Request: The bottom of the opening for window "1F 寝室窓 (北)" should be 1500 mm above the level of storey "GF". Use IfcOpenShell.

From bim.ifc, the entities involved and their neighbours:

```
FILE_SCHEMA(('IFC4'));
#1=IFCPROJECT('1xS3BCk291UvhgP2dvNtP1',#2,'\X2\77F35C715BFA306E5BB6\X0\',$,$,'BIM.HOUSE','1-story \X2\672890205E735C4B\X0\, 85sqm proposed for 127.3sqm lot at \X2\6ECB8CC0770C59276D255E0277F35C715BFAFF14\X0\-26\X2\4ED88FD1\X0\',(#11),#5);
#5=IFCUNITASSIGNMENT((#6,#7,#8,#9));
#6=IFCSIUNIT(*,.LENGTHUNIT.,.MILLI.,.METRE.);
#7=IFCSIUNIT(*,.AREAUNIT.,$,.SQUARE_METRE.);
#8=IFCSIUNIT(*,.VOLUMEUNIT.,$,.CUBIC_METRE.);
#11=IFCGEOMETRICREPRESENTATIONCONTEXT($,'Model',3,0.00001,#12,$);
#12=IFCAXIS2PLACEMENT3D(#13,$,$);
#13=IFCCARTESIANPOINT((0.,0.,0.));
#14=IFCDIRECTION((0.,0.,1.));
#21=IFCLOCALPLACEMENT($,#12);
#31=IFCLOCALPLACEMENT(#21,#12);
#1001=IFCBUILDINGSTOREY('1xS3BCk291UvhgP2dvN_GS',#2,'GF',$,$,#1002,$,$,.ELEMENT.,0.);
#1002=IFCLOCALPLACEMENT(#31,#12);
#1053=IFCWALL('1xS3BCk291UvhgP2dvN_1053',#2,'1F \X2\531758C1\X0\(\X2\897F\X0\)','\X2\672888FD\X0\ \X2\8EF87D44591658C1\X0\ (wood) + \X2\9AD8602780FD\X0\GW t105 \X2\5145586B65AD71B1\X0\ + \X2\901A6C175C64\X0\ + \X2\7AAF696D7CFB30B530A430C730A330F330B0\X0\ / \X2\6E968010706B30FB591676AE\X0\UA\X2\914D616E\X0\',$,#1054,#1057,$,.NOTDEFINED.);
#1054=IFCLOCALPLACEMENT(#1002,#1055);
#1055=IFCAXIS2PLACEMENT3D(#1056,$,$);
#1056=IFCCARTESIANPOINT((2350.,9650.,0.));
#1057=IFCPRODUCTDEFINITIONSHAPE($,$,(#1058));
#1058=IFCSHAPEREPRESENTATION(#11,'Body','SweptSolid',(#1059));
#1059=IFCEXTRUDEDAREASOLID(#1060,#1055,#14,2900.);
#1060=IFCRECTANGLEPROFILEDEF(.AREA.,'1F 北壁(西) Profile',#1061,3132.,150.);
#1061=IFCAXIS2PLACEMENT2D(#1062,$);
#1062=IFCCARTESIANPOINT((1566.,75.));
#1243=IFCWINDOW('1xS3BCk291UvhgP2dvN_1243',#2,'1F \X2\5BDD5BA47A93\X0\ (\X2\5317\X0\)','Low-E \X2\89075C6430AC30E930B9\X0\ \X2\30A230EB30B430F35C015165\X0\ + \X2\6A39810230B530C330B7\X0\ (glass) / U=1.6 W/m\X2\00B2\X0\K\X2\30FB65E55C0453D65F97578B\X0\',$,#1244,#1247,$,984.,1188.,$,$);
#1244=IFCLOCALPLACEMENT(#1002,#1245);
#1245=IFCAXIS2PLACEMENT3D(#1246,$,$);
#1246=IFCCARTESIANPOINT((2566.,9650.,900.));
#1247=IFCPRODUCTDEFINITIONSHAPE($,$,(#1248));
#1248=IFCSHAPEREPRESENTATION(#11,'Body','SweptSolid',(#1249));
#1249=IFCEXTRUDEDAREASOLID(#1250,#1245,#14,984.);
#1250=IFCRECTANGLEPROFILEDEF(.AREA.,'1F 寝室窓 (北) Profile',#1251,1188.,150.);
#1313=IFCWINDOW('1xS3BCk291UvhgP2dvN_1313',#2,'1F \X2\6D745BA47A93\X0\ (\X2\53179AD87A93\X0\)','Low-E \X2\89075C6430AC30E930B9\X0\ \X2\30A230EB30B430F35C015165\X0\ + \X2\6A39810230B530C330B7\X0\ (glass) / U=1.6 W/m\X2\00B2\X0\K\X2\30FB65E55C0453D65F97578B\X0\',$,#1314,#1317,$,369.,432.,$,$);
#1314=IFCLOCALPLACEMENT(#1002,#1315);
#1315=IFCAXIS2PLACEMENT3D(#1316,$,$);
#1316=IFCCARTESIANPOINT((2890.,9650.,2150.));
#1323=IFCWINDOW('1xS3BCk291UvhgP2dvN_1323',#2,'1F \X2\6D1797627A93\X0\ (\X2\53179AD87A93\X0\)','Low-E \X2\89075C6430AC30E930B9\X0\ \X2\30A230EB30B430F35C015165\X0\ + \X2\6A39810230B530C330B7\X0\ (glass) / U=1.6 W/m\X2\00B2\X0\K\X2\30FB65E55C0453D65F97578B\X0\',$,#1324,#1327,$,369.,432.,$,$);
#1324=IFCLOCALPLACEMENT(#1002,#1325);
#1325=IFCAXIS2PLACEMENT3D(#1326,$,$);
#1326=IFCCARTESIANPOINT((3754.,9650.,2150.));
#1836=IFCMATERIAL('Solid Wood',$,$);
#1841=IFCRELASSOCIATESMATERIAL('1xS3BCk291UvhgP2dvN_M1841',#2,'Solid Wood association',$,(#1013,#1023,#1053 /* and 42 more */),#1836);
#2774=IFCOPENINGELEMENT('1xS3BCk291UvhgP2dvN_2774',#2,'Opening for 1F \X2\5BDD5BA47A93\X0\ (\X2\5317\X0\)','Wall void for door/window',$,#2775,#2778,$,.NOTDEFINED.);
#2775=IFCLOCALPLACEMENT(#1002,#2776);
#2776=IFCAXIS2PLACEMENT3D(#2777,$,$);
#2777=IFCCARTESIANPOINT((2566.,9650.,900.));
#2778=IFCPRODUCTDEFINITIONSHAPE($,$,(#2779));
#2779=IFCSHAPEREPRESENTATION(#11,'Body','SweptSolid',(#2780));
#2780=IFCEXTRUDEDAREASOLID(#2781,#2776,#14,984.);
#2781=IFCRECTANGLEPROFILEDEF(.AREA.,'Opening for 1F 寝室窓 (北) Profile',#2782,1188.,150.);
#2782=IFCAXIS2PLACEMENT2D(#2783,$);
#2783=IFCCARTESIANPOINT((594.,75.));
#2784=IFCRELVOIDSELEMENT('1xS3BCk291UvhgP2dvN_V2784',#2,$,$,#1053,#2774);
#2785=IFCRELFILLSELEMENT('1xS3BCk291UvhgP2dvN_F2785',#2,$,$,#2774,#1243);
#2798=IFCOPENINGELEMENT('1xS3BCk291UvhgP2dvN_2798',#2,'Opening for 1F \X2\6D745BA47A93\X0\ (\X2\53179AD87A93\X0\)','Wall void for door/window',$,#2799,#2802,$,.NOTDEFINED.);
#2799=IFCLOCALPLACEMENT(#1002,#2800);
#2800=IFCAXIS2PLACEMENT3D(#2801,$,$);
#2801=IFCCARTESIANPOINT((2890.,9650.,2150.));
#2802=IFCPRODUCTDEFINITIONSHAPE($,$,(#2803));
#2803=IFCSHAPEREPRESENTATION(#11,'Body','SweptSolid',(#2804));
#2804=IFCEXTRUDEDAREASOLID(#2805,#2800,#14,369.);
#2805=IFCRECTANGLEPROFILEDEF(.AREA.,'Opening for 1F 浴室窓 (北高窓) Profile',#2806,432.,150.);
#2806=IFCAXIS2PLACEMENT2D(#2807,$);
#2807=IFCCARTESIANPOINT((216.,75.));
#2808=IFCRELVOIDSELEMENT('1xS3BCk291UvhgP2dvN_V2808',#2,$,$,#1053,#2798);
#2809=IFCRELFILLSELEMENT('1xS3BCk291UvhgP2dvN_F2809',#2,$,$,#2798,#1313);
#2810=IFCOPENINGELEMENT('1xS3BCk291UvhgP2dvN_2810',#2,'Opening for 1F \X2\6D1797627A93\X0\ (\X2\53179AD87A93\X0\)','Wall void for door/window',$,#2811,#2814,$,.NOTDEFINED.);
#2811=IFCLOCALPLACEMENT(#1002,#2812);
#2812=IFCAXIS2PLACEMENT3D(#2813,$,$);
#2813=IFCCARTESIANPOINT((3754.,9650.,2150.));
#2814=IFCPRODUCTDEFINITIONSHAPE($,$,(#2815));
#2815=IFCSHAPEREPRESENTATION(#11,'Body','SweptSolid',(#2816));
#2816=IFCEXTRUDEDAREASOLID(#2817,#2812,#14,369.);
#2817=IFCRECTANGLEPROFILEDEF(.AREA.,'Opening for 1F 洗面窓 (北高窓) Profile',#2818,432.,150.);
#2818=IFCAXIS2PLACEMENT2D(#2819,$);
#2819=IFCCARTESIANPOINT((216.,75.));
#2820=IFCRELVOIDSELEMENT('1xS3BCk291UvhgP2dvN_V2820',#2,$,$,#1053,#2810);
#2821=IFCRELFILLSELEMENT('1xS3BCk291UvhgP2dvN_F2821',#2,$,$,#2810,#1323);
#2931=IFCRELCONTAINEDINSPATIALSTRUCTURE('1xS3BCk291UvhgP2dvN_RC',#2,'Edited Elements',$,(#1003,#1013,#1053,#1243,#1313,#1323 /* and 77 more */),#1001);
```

```python
import numpy as np
import ifcopenshell
import ifcopenshell.api.geometry
import ifcopenshell.geom
import ifcopenshell.util.element
import ifcopenshell.util.placement
import ifcopenshell.util.shape
import ifcopenshell.util.unit

model = ifcopenshell.open("bim.ifc")
unit_scale = ifcopenshell.util.unit.calculate_unit_scale(model)

window = model.by_guid("1xS3BCk291UvhgP2dvN_1243")
opening = window.FillsVoids[0].RelatingOpeningElement
storey = ifcopenshell.util.element.get_container(window, ifc_class="IfcBuildingStorey")
level = ifcopenshell.util.placement.get_local_placement(storey.ObjectPlacement)[2, 3]

# The opening's origin need not be at the sill, so measure its lowest point.
shape = ifcopenshell.geom.create_shape(ifcopenshell.geom.settings(), opening)
bottom = ifcopenshell.util.shape.get_shape_bottom_elevation(shape, shape.geometry) / unit_scale
dz = level + 1.5 / unit_scale - bottom

shift = np.array([0.0, 0.0, dz])
# The window is not placed relative to its opening, so move both.
for product in (opening, window):
    matrix = ifcopenshell.util.placement.get_local_placement(product.ObjectPlacement)
    matrix[:3, 3] += shift
    ifcopenshell.api.geometry.edit_object_placement(model, product=product, matrix=matrix, is_si=False)

print(f"moved by {dz * unit_scale:+.3f} m")

model.write("bim_v2.ifc")
```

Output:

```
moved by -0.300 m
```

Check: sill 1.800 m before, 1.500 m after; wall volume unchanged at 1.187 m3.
